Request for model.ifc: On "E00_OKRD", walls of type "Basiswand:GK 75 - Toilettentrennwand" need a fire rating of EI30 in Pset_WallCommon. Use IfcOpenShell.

First a look at what the model holds.

```python
import ifcopenshell
import ifcopenshell.util.element

model = ifcopenshell.open("model.ifc")
print(model.schema)
storey = next(s for s in model.by_type("IfcBuildingStorey") if s.Name == "E00_OKRD")
walls = [e for e in ifcopenshell.util.element.get_decomposition(storey) if e.is_a("IfcWall")]
seen = {}
for e in walls:
    element_type = ifcopenshell.util.element.get_type(e)
    key = (element_type.Name if element_type != e and element_type else None, ifcopenshell.util.element.get_pset(e, "Pset_WallCommon", "FireRating"))
    seen[key] = seen.get(key, 0) + 1
for (name, value), count in sorted(seen.items(), key=str):
    print(count, "x", name, "|", value)
```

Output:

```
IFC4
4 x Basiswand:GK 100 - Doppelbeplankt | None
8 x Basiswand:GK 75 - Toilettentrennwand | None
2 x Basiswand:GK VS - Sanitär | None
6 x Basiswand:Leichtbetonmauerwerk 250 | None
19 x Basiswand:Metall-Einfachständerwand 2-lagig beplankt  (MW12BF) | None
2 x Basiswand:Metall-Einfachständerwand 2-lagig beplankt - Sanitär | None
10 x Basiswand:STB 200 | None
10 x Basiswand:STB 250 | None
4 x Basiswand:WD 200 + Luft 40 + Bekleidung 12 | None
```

```python
import ifcopenshell
import ifcopenshell.api.pset
import ifcopenshell.util.element

model = ifcopenshell.open("model.ifc")

storey = next(s for s in model.by_type("IfcBuildingStorey") if s.Name == "E00_OKRD")
walls = [e for e in ifcopenshell.util.element.get_decomposition(storey) if e.is_a("IfcWall")]

count = 0
for e in walls:
    element_type = ifcopenshell.util.element.get_type(e)
    if element_type in (None, e) or element_type.Name != "Basiswand:GK 75 - Toilettentrennwand":
        continue
    # add_pset returns the element's existing set when there is one.
    pset = ifcopenshell.api.pset.add_pset(model, product=e, name="Pset_WallCommon")
    ifcopenshell.api.pset.edit_pset(model, pset=pset, properties={"FireRating": "EI30"})
    count += 1

print(count, "walls updated")

model.write("model_edited.ifc")
```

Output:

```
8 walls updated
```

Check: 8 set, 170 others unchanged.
